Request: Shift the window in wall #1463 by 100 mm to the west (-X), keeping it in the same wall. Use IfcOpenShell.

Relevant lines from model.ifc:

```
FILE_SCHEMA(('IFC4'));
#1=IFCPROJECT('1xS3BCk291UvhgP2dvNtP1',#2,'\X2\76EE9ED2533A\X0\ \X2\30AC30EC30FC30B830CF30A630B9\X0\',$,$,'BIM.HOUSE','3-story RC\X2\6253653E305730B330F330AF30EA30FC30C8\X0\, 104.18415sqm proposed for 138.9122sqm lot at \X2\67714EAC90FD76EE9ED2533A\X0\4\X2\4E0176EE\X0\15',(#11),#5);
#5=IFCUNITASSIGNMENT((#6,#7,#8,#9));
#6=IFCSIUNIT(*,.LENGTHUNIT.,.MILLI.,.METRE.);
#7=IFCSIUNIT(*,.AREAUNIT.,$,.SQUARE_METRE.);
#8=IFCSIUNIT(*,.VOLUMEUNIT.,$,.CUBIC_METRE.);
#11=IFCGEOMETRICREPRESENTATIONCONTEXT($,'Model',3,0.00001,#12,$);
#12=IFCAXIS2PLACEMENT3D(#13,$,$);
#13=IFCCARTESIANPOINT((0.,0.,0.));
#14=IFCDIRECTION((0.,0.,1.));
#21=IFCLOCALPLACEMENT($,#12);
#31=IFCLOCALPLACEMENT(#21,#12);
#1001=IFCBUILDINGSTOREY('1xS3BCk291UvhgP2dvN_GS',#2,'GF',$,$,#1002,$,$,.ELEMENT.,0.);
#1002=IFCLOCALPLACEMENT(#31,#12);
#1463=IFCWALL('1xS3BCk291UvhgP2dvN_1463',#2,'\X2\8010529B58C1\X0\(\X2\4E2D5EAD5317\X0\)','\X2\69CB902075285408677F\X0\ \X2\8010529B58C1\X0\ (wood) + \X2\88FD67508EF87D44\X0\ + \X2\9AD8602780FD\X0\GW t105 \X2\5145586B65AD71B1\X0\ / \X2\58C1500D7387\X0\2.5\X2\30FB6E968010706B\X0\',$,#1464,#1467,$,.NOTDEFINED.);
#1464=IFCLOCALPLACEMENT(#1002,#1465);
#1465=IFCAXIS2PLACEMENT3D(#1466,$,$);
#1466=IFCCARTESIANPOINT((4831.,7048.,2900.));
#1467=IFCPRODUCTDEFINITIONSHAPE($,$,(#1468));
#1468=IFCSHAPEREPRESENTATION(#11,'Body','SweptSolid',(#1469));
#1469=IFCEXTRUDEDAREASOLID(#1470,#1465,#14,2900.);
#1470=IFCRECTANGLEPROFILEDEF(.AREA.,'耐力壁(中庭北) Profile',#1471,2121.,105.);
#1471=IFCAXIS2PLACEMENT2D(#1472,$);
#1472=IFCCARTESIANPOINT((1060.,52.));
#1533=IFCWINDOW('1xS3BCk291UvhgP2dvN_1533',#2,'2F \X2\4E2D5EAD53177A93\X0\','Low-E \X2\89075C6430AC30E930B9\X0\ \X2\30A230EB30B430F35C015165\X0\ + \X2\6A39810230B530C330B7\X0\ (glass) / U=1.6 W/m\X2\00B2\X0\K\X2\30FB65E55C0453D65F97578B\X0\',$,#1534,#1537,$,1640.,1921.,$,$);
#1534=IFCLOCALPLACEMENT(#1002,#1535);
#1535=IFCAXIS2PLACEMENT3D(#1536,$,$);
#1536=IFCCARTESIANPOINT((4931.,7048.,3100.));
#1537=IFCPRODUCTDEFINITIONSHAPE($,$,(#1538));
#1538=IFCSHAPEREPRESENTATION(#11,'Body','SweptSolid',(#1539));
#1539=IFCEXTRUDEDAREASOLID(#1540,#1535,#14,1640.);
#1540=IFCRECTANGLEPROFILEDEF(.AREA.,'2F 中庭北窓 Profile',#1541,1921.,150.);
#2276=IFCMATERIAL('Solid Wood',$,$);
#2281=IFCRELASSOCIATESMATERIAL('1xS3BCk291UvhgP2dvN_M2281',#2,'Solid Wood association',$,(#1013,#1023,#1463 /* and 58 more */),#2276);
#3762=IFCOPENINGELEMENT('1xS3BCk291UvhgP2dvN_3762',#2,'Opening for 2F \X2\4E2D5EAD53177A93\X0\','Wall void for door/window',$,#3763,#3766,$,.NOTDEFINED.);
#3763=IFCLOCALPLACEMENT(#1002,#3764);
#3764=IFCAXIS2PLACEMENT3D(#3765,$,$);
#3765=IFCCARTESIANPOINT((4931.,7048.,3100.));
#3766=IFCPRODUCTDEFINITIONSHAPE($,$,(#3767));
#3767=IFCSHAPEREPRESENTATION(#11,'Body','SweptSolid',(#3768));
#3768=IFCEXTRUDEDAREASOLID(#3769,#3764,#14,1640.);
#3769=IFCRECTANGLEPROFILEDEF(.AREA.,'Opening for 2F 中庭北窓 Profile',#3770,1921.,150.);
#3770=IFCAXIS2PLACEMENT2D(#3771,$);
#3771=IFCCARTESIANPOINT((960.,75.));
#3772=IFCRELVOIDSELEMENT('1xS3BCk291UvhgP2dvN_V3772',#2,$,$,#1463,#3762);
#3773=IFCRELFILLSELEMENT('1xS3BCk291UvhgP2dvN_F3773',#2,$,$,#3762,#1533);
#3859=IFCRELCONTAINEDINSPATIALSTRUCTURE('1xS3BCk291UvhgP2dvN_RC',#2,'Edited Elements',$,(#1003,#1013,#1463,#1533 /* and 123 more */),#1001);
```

```python
import ifcopenshell
import ifcopenshell.api.geometry
import ifcopenshell.util.placement
import ifcopenshell.util.unit

model = ifcopenshell.open("model.ifc")
unit_scale = ifcopenshell.util.unit.calculate_unit_scale(model)

window = model.by_guid("1xS3BCk291UvhgP2dvN_1533")
opening = window.FillsVoids[0].RelatingOpeningElement
wall = opening.VoidsElements[0].RelatingBuildingElement

wall_matrix = ifcopenshell.util.placement.get_local_placement(wall.ObjectPlacement)
shift = wall_matrix[:3, 0] * -0.1 / unit_scale
before = ifcopenshell.util.placement.get_local_placement(window.ObjectPlacement)[:3, 3].copy()

# The window is not placed relative to its opening, so move both.
for product in (opening, window):
    matrix = ifcopenshell.util.placement.get_local_placement(product.ObjectPlacement)
    matrix[:3, 3] += shift
    ifcopenshell.api.geometry.edit_object_placement(model, product=product, matrix=matrix, is_si=False)

after = ifcopenshell.util.placement.get_local_placement(window.ObjectPlacement)[:3, 3]
print("window moved by", (after - before).round(3) + 0.0)

model.write("model-out.ifc")
```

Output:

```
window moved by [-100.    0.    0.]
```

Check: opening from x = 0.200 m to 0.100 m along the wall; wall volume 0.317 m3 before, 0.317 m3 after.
